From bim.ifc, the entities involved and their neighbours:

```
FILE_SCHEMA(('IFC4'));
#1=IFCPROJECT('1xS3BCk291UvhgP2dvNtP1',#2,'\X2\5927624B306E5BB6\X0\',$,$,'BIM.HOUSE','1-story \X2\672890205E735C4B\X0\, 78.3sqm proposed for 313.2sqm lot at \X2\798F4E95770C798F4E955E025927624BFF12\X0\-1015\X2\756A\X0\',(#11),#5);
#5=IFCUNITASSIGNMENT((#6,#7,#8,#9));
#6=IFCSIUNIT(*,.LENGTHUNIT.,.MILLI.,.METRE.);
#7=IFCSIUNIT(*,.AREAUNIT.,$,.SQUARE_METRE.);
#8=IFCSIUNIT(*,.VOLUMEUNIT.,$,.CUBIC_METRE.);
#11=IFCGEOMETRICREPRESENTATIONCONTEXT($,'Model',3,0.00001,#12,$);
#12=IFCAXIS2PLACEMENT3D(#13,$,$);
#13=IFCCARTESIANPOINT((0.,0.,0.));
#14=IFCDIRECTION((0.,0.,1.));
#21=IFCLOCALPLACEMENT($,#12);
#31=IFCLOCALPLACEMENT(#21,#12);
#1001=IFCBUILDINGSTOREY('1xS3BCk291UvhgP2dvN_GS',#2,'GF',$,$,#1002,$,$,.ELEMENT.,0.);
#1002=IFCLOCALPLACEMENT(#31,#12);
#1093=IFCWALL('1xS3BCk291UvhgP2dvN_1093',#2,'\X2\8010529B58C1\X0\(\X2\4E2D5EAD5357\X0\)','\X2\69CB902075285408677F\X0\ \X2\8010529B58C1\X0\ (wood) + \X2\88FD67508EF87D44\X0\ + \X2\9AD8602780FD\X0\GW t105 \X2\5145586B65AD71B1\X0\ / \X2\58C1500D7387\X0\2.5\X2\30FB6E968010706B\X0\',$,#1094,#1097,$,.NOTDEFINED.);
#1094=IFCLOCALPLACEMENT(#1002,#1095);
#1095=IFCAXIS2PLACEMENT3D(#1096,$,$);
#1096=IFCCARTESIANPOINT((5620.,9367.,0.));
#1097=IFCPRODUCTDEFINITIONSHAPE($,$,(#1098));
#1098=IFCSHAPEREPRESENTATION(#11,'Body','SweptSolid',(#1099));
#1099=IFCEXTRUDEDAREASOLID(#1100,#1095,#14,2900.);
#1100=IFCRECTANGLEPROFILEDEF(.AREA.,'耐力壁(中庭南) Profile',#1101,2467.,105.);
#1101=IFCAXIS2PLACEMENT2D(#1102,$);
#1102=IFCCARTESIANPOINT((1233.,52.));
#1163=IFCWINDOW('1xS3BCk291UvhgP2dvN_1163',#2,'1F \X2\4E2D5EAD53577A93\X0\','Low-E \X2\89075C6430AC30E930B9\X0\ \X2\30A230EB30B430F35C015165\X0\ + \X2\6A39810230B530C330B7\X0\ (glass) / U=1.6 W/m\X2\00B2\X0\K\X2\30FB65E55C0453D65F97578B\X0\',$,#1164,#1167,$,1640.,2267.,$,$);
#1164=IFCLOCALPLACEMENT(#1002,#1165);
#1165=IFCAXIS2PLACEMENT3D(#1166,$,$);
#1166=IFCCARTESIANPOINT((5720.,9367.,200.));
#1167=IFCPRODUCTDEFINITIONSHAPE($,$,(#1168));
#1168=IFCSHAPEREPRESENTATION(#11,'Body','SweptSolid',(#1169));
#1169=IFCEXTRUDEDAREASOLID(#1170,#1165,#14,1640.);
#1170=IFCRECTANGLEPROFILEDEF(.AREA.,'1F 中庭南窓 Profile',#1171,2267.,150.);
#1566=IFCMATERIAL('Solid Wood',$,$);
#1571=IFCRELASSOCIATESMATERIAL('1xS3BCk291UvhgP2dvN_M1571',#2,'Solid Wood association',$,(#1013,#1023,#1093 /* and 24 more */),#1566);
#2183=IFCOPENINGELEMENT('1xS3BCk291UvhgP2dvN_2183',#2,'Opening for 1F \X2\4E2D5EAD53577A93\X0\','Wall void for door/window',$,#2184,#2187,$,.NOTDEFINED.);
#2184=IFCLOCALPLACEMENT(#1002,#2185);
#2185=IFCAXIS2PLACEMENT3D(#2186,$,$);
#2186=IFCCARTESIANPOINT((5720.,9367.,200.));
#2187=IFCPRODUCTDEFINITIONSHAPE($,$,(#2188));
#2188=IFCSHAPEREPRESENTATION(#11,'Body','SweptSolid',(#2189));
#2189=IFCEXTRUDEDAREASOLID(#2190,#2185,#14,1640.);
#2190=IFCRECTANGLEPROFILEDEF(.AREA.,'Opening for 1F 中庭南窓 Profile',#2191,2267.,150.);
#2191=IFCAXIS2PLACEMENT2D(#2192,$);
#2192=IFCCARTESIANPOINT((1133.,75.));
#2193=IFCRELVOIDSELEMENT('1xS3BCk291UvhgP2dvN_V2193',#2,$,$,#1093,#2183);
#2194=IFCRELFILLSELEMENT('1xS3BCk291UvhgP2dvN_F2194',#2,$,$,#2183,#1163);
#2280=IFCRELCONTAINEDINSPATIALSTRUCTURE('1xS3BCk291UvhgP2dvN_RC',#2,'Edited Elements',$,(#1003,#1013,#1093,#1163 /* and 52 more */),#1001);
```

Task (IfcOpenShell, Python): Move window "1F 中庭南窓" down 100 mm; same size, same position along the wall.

```python
import numpy as np
import ifcopenshell
import ifcopenshell.api.geometry
import ifcopenshell.util.placement
import ifcopenshell.util.unit

model = ifcopenshell.open("bim.ifc")
unit_scale = ifcopenshell.util.unit.calculate_unit_scale(model)

window = model.by_guid("1xS3BCk291UvhgP2dvN_1163")
opening = window.FillsVoids[0].RelatingOpeningElement
dz = -0.1 / unit_scale

shift = np.array([0.0, 0.0, dz])
# The window is not placed relative to its opening, so move both.
for product in (opening, window):
    matrix = ifcopenshell.util.placement.get_local_placement(product.ObjectPlacement)
    matrix[:3, 3] += shift
    ifcopenshell.api.geometry.edit_object_placement(model, product=product, matrix=matrix, is_si=False)

print(f"moved by {dz * unit_scale:+.3f} m")

model.write("bim_v2.ifc")
```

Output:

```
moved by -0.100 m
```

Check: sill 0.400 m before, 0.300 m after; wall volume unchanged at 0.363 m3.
